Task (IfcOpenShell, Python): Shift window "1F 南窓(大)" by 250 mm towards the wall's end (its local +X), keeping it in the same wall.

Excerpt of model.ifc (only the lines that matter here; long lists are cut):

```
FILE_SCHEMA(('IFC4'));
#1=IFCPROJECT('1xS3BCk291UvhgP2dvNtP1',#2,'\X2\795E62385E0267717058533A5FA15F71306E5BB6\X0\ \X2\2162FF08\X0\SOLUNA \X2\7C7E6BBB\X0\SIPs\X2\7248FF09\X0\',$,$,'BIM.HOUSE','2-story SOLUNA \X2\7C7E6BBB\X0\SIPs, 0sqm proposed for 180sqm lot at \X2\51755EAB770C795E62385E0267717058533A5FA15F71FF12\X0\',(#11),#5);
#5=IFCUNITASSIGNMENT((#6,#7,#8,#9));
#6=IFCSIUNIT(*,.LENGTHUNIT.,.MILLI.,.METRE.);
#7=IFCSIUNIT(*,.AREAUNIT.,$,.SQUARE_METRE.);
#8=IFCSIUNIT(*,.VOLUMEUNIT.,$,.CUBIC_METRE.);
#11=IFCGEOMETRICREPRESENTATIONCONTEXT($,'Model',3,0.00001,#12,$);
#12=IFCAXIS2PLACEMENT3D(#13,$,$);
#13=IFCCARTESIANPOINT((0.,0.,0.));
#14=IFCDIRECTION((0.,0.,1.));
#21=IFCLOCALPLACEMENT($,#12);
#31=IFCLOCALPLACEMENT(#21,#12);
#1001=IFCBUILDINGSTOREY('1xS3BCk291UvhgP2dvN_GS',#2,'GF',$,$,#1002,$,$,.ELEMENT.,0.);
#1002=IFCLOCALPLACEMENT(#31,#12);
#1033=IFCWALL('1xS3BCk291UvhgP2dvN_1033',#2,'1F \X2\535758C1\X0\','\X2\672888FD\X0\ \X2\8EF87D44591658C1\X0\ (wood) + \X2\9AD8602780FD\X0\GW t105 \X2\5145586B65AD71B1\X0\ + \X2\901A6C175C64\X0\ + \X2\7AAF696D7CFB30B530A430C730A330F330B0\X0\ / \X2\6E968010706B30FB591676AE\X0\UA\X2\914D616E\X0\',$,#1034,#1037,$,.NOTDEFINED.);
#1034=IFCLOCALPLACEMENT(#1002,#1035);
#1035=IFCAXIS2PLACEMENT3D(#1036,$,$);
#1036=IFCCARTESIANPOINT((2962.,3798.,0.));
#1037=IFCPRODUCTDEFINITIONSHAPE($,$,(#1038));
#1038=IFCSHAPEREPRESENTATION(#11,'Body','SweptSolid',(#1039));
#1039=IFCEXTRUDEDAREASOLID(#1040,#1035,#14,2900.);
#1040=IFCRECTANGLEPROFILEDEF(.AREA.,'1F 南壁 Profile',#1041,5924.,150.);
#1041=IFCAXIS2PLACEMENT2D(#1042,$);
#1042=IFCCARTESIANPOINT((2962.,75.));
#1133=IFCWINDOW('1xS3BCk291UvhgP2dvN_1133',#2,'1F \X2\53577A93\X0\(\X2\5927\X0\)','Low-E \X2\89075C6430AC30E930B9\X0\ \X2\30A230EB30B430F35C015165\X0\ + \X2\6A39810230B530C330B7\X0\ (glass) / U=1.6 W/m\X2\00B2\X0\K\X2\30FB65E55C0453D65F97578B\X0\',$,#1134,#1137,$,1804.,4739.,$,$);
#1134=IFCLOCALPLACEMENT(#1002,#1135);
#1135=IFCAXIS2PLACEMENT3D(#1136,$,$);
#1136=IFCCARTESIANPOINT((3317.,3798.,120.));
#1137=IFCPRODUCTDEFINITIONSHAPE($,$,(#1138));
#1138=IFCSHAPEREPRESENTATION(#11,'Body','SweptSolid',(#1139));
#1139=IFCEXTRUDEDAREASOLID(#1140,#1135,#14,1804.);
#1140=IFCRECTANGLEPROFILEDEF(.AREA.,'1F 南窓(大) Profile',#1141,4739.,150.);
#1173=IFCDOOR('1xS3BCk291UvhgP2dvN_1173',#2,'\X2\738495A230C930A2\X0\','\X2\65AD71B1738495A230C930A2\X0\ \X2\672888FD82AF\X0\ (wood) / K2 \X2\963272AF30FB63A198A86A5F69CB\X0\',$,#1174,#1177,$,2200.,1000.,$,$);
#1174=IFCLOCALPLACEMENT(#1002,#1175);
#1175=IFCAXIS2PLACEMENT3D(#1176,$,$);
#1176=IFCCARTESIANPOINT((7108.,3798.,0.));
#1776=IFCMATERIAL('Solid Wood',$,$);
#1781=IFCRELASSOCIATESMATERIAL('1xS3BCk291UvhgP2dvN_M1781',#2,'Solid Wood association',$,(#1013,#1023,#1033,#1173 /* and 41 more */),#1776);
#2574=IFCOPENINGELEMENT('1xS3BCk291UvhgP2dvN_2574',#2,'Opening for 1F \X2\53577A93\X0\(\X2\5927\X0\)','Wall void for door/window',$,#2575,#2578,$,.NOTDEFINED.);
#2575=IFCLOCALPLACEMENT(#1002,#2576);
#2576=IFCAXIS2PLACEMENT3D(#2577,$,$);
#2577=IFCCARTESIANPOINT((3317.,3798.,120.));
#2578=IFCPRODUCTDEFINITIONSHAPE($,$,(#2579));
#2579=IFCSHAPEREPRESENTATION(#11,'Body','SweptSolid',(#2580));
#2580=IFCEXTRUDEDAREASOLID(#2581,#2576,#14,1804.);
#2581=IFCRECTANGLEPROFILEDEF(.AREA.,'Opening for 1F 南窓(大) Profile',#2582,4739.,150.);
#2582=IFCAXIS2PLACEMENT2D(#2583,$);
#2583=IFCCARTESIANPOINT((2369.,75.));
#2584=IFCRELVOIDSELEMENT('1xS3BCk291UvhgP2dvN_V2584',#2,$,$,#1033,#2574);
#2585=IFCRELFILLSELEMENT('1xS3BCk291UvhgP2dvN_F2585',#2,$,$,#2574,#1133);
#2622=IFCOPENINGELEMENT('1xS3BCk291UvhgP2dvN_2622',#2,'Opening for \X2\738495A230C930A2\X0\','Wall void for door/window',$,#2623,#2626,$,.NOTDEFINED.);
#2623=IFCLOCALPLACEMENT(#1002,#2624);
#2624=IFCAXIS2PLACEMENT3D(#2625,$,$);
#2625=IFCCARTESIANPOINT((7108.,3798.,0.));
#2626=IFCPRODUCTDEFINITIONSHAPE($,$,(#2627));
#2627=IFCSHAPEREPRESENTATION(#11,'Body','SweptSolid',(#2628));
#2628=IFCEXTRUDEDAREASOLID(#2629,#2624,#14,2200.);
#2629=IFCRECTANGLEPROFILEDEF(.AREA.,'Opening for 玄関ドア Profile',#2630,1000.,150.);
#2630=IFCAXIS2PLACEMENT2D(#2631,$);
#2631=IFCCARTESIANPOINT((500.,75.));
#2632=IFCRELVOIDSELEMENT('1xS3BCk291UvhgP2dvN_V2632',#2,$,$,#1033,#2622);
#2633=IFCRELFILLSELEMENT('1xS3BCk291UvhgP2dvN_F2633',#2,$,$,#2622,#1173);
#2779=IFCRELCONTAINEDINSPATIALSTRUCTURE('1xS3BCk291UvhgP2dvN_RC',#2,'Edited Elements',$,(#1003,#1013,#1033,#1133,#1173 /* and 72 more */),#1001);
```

```python
import ifcopenshell
import ifcopenshell.api.geometry
import ifcopenshell.util.placement
import ifcopenshell.util.unit

model = ifcopenshell.open("model.ifc")
unit_scale = ifcopenshell.util.unit.calculate_unit_scale(model)

window = model.by_id(1133)
opening = window.FillsVoids[0].RelatingOpeningElement
wall = opening.VoidsElements[0].RelatingBuildingElement

wall_matrix = ifcopenshell.util.placement.get_local_placement(wall.ObjectPlacement)
shift = wall_matrix[:3, 0] * 0.25 / unit_scale
before = ifcopenshell.util.placement.get_local_placement(window.ObjectPlacement)[:3, 3].copy()

# The window is not placed relative to its opening, so move both.
for product in (opening, window):
    matrix = ifcopenshell.util.placement.get_local_placement(product.ObjectPlacement)
    matrix[:3, 3] += shift
    ifcopenshell.api.geometry.edit_object_placement(model, product=product, matrix=matrix, is_si=False)

after = ifcopenshell.util.placement.get_local_placement(window.ObjectPlacement)[:3, 3]
print("window moved by", (after - before).round(3) + 0.0)

model.write("model_updated.ifc")
```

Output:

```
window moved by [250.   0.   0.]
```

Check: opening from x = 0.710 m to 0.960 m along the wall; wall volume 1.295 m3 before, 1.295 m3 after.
